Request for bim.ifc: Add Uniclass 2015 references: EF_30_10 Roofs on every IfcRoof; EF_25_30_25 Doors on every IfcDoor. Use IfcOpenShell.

First a look at what the model holds.

```python
import ifcopenshell

model = ifcopenshell.open("bim.ifc")
print(model.schema)
print("classifications:", [c.Name for c in model.by_type("IfcClassification")])
for ifc_class in ("IfcDoor", "IfcRoof", "IfcStair", "IfcWall", "IfcWindow"):
    print(ifc_class, len(model.by_type(ifc_class)))
```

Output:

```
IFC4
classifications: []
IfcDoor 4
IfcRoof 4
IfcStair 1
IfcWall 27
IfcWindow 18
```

```python
import ifcopenshell
import ifcopenshell.api.classification

model = ifcopenshell.open("bim.ifc")

system = ifcopenshell.api.classification.add_classification(model, classification="Uniclass 2015")

codes = {
    "IfcRoof": ("EF_30_10", "Roofs"),
    "IfcDoor": ("EF_25_30_25", "Doors"),
}
for ifc_class, (code, name) in codes.items():
    products = model.by_type(ifc_class)
    ifcopenshell.api.classification.add_reference(
        model, products=products, classification=system, identification=code, name=name
    )
    print(code, len(products))

model.write("bim_rev.ifc")
```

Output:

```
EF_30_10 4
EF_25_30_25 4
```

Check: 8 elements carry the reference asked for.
